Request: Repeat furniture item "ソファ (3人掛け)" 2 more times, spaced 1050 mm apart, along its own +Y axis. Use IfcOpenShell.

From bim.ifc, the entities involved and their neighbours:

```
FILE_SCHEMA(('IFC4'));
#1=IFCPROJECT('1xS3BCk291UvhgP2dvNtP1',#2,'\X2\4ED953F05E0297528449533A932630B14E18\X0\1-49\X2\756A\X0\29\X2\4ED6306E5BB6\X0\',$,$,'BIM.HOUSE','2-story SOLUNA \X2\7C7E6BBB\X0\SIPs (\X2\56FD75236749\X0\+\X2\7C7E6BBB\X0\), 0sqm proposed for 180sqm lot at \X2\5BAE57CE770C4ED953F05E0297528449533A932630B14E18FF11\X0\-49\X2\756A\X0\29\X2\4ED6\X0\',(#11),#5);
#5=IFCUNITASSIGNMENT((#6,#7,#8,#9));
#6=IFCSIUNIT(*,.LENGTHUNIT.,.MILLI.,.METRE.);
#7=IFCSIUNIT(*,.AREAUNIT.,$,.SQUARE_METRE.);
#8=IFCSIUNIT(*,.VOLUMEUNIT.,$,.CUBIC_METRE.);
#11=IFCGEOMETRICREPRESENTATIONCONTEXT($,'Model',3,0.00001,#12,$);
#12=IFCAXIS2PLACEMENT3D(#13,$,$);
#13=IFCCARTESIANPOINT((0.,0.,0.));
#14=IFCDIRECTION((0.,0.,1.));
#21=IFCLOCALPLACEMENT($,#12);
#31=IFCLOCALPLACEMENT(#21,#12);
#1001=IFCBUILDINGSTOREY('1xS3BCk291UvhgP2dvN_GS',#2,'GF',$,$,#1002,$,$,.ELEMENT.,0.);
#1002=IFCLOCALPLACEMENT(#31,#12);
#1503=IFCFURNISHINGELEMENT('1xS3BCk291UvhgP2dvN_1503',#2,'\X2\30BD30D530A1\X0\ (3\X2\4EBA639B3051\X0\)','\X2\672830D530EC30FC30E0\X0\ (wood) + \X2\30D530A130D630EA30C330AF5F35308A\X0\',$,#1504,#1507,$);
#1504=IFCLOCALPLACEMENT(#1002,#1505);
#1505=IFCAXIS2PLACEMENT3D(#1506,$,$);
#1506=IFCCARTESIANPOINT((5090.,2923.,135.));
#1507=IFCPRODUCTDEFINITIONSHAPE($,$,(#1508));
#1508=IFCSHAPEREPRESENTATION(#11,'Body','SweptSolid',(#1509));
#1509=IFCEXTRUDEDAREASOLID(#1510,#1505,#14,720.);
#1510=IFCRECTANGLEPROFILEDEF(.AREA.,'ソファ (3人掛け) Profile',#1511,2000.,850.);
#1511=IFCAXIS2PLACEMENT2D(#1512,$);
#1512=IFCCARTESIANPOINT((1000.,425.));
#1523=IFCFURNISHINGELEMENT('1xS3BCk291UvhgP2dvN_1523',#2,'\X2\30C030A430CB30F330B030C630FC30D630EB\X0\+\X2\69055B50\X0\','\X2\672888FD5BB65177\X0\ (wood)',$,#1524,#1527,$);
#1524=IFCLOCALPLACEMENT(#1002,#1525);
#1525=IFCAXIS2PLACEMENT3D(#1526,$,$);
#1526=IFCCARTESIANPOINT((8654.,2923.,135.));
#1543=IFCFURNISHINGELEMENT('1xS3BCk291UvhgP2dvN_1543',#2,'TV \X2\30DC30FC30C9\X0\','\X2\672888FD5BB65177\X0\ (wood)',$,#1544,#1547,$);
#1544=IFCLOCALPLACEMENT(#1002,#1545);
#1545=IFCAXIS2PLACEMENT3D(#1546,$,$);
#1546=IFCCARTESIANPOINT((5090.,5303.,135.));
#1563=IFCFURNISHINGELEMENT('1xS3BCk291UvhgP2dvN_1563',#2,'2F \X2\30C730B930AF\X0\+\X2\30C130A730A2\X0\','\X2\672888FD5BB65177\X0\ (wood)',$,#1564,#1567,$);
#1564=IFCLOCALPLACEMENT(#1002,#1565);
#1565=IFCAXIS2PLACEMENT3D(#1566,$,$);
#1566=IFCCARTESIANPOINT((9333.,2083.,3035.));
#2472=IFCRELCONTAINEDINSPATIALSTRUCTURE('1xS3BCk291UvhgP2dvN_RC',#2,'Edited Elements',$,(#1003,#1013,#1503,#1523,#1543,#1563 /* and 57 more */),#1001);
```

```python
import ifcopenshell
import ifcopenshell.api.geometry
import ifcopenshell.api.root
import ifcopenshell.util.element
import ifcopenshell.util.placement
import ifcopenshell.util.unit

model = ifcopenshell.open("bim.ifc")
unit_scale = ifcopenshell.util.unit.calculate_unit_scale(model)


def reuse_history(source, copy):
    """copy_class also copies each property set's owner history, people and application; keep the originals."""
    for rel in copy.IsDefinedBy:
        if rel.is_a("IfcRelDefinesByProperties") and (history := rel.RelatingPropertyDefinition.OwnerHistory):
            rel.RelatingPropertyDefinition.OwnerHistory = source.OwnerHistory
            ifcopenshell.util.element.remove_deep2(model, history)


source = model.by_guid("1xS3BCk291UvhgP2dvN_1503")
base = ifcopenshell.util.placement.get_local_placement(source.ObjectPlacement)
step = base[:3, 1] * 1.05 / unit_scale

for i in range(1, 3):
    copy = ifcopenshell.api.root.copy_class(model, product=source)
    copy.Representation = ifcopenshell.util.element.copy_deep(
        model, source.Representation, exclude=["IfcGeometricRepresentationContext", "IfcRepresentationMap"]
    )
    reuse_history(source, copy)
    matrix = base.copy()
    matrix[:3, 3] += i * step
    print("added at", matrix[:3, 3].round(3) + 0.0)
    ifcopenshell.api.geometry.edit_object_placement(model, product=copy, matrix=matrix, is_si=False)

model.write("bim-out.ifc")
```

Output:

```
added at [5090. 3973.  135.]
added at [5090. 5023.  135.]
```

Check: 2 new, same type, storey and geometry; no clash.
